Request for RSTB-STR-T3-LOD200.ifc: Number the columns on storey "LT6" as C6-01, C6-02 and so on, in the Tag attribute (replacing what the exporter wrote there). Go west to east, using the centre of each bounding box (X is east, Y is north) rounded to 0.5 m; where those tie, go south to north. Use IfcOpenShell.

First a look at what the model holds.

```python
import ifcopenshell
import ifcopenshell.util.element
import ifcopenshell.util.placement

model = ifcopenshell.open("RSTB-STR-T3-LOD200.ifc")
print(model.schema)
storey = next(s for s in model.by_type("IfcBuildingStorey") if s.Name == "LT6")
columns = [e for e in ifcopenshell.util.element.get_decomposition(storey) if e.is_a("IfcColumn")]
for e in sorted(columns, key=lambda e: e.id()):
    origin = ifcopenshell.util.placement.get_local_placement(e.ObjectPlacement)[:3, 3]
    print(e.id(), e.Tag, e.Name, origin.round(2) + 0.0, sep=" | ")
```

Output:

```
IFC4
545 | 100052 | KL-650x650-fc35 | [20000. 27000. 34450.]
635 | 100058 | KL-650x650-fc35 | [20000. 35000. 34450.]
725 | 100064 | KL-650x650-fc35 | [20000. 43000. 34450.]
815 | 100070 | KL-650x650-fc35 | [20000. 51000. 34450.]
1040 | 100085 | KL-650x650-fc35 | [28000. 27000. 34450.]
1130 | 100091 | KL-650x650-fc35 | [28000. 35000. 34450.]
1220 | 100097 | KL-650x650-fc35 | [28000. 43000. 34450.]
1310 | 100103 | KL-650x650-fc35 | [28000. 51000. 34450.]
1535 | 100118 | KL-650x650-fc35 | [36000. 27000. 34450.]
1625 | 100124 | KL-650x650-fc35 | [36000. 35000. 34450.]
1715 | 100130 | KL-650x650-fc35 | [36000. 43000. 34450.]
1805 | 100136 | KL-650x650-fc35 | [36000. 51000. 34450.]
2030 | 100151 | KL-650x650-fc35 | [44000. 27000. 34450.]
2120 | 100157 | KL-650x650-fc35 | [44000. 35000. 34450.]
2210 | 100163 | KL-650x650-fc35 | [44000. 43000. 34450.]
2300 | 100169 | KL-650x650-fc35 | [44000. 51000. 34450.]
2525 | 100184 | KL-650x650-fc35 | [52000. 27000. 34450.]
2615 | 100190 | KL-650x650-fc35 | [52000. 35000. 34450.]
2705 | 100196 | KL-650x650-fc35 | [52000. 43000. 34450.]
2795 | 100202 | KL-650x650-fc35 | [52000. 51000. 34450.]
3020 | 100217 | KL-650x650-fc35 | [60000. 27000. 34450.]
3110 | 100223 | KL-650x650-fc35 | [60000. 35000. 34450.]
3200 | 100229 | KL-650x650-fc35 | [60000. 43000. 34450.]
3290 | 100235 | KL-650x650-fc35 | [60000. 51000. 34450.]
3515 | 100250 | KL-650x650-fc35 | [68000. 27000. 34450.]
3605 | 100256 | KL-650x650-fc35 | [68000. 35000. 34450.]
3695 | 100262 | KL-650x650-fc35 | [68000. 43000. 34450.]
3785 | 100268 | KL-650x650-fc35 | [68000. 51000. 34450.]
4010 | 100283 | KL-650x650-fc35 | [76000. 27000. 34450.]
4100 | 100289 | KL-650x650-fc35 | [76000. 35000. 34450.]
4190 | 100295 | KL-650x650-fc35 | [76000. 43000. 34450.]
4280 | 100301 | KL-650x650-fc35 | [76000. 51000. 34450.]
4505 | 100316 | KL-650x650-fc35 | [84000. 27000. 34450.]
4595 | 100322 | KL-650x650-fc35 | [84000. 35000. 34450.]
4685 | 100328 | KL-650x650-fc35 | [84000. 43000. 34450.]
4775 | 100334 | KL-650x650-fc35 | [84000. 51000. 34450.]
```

```python
import ifcopenshell
import ifcopenshell.geom
import ifcopenshell.util.element
import ifcopenshell.util.shape

model = ifcopenshell.open("RSTB-STR-T3-LOD200.ifc")
settings = ifcopenshell.geom.settings()
settings.set("use-world-coords", True)


def centre(element):
    shape = ifcopenshell.geom.create_shape(settings, element)
    return ifcopenshell.util.shape.get_bbox_centroid(shape.geometry)


storey = next(s for s in model.by_type("IfcBuildingStorey") if s.Name == "LT6")
columns = [e for e in ifcopenshell.util.element.get_decomposition(storey) if e.is_a("IfcColumn")]

# Insertion points can sit at a corner or the storey origin, so sort by the geometry (in metres).
centres = {e: centre(e) for e in columns}
columns.sort(key=lambda e: (round(centres[e][0] / 0.5), centres[e][1]))

for i, e in enumerate(columns, start=1):
    number = f"C6-{i:02d}"
    e.Tag = number
    print(e.id(), number)

model.write("RSTB-STR-T3-LOD200_v2.ifc")
```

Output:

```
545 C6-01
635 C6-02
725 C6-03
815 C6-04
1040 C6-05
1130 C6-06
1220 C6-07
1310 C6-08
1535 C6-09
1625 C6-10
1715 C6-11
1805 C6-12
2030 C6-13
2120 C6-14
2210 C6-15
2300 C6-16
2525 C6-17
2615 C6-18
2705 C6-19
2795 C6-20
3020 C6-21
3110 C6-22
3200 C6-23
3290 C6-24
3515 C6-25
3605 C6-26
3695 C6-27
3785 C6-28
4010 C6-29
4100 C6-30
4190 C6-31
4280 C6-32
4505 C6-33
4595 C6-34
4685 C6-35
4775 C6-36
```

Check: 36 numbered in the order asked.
